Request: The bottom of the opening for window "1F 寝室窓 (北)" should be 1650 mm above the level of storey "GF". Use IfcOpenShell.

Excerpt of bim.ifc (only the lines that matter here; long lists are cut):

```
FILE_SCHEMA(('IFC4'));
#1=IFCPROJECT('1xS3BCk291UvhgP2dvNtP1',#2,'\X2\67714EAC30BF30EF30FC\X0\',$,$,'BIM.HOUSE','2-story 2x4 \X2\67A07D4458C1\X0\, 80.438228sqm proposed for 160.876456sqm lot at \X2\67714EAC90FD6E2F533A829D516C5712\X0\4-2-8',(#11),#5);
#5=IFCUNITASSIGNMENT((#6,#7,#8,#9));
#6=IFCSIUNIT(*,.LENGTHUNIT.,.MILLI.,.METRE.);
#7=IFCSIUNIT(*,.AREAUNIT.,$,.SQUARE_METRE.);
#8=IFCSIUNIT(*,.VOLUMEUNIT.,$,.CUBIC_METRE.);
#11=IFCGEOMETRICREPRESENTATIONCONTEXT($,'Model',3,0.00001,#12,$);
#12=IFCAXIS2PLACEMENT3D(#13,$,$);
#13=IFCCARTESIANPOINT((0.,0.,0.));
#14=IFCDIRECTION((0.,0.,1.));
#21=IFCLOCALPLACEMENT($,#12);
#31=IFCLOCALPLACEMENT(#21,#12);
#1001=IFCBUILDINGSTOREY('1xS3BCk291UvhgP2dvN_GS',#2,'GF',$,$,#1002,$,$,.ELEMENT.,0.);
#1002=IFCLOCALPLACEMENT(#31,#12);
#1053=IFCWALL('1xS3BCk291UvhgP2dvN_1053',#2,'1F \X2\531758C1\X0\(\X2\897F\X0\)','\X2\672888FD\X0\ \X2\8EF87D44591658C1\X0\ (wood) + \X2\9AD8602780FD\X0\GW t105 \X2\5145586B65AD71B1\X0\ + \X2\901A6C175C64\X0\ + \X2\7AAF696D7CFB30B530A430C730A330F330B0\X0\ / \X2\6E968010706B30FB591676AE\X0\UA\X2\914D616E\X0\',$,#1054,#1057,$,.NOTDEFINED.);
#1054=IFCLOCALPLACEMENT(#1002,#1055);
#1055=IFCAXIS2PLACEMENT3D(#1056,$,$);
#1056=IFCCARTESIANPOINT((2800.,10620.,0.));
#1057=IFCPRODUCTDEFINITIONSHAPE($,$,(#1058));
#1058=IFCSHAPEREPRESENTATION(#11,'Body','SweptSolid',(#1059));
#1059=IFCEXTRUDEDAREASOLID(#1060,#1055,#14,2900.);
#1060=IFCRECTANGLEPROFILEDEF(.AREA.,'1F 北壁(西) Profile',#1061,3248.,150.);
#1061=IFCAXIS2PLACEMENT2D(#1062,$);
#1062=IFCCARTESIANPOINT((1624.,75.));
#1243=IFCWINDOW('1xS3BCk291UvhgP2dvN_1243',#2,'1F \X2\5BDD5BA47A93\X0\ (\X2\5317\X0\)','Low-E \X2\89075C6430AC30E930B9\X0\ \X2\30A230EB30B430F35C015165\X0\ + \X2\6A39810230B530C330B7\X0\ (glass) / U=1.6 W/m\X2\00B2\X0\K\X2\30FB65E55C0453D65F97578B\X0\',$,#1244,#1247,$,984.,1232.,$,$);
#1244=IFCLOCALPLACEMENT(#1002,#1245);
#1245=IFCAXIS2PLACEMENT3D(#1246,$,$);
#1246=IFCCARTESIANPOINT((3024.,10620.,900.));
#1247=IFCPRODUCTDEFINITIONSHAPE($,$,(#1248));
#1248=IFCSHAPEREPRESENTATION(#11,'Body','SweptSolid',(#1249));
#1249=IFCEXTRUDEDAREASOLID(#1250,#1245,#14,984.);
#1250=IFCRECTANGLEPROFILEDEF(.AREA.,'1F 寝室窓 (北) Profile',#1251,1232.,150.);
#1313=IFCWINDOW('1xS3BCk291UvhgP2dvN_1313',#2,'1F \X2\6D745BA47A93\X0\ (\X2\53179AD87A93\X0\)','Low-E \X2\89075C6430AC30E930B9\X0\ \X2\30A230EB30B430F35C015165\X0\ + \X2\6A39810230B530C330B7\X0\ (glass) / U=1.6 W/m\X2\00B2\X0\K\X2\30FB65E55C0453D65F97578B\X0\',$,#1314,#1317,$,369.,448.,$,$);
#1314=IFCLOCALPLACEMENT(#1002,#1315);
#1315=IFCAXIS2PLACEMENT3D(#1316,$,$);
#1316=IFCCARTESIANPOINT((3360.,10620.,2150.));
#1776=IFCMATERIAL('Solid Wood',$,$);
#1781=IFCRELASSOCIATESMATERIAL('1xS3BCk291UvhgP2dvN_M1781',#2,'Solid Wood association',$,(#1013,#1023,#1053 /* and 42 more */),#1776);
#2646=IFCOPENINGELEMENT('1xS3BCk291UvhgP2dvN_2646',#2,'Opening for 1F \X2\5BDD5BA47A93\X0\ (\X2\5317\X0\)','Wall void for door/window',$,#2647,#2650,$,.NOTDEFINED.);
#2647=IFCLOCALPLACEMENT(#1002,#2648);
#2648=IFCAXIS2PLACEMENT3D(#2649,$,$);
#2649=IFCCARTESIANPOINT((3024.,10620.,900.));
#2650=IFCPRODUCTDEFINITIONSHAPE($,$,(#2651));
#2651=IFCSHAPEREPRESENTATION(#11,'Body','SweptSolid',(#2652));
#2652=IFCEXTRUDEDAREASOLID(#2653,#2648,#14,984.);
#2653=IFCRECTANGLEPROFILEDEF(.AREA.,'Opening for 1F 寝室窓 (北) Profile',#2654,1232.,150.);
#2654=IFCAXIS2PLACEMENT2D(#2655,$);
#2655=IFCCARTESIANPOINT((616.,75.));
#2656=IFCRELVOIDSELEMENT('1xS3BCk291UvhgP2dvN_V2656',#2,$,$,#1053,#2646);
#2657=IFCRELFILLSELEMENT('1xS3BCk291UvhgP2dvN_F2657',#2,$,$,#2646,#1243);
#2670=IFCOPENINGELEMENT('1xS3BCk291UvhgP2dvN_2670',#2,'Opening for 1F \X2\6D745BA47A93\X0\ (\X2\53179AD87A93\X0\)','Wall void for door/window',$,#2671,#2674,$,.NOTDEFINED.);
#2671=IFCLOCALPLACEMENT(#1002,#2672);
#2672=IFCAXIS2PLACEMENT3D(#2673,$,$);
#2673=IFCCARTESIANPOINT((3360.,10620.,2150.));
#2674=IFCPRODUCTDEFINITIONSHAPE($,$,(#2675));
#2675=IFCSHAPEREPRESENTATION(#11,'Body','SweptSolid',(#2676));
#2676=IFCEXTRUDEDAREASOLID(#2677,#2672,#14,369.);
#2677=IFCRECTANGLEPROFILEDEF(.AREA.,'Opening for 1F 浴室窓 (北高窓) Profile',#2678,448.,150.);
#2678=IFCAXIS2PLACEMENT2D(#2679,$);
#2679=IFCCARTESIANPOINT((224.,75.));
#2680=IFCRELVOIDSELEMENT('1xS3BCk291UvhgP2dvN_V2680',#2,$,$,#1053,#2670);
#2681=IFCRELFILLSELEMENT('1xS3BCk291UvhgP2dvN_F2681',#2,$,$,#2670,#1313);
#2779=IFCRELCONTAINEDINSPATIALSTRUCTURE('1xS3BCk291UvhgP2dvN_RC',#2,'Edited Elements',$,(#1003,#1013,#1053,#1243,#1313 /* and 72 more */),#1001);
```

```python
import numpy as np
import ifcopenshell
import ifcopenshell.api.geometry
import ifcopenshell.geom
import ifcopenshell.util.element
import ifcopenshell.util.placement
import ifcopenshell.util.shape
import ifcopenshell.util.unit

model = ifcopenshell.open("bim.ifc")
unit_scale = ifcopenshell.util.unit.calculate_unit_scale(model)

window = model.by_guid("1xS3BCk291UvhgP2dvN_1243")
opening = window.FillsVoids[0].RelatingOpeningElement
storey = ifcopenshell.util.element.get_container(window, ifc_class="IfcBuildingStorey")
level = ifcopenshell.util.placement.get_local_placement(storey.ObjectPlacement)[2, 3]

# The opening's origin need not be at the sill, so measure its lowest point.
shape = ifcopenshell.geom.create_shape(ifcopenshell.geom.settings(), opening)
bottom = ifcopenshell.util.shape.get_shape_bottom_elevation(shape, shape.geometry) / unit_scale
dz = level + 1650.0 - bottom

shift = np.array([0.0, 0.0, dz])
# The window is not placed relative to its opening, so move both.
for product in (opening, window):
    matrix = ifcopenshell.util.placement.get_local_placement(product.ObjectPlacement)
    matrix[:3, 3] += shift
    ifcopenshell.api.geometry.edit_object_placement(model, product=product, matrix=matrix, is_si=False)

print(f"moved by {dz * unit_scale:+.3f} m")

model.write("bim_v2.ifc")
```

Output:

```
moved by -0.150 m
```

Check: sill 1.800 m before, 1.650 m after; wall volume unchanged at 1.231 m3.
